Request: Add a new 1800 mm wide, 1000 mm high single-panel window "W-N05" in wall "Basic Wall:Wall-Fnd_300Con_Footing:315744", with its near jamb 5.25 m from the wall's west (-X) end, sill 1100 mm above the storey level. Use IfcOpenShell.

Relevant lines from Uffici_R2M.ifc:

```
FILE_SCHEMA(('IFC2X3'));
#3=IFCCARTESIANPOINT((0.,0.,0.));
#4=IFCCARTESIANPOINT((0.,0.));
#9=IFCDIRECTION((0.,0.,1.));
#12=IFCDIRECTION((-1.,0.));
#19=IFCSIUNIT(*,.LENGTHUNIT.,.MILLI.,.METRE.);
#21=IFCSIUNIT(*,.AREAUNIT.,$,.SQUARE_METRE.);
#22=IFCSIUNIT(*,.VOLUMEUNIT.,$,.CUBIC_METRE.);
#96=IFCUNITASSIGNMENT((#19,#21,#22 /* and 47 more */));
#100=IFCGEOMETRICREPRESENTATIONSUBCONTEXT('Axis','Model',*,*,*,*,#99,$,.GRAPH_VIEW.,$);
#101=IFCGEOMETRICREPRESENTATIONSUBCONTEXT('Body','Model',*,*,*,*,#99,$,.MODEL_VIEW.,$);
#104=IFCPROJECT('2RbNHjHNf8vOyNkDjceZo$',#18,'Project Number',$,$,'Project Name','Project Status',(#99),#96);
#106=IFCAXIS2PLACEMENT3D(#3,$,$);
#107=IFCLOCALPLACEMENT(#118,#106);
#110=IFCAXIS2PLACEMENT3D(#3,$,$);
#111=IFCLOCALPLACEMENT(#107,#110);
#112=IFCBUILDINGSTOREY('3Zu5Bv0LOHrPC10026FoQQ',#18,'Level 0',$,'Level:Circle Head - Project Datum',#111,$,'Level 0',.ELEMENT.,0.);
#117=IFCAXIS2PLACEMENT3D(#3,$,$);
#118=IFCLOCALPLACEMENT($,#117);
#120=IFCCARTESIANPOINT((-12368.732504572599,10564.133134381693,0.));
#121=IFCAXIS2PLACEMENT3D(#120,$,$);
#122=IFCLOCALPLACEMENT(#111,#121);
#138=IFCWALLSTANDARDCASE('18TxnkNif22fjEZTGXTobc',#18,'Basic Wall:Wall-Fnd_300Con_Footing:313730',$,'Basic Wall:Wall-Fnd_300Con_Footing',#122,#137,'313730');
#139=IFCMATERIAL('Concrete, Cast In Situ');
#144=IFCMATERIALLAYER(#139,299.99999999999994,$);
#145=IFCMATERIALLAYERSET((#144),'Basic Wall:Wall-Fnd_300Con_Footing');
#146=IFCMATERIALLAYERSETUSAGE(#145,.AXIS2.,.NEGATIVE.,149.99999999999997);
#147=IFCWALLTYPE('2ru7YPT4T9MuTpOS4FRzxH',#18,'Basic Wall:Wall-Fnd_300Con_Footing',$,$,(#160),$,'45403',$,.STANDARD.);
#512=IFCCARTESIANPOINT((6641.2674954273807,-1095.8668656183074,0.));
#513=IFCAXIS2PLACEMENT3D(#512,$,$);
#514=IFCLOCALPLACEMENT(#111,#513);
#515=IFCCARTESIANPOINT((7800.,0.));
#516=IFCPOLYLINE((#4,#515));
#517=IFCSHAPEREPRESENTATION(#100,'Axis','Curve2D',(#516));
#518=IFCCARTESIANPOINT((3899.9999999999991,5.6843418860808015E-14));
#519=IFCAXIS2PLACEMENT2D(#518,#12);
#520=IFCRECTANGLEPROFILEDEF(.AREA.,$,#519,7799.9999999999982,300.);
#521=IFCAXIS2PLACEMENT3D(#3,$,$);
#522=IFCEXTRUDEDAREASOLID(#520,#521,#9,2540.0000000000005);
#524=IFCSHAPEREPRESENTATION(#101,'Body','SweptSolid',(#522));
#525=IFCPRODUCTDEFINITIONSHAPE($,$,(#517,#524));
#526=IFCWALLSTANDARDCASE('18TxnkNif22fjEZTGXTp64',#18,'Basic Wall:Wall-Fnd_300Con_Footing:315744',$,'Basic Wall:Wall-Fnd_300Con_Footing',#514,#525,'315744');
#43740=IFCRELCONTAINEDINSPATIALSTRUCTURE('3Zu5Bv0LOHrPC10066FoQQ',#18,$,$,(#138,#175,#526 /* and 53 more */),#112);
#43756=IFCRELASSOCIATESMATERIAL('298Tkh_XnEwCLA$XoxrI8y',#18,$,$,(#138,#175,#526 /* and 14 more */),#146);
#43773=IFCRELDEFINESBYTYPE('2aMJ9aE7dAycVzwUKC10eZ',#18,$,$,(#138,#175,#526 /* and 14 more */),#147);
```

```python
import numpy as np
import ifcopenshell
import ifcopenshell.api.feature
import ifcopenshell.api.geometry
import ifcopenshell.api.root
import ifcopenshell.api.spatial
import ifcopenshell.api.type
import ifcopenshell.geom
import ifcopenshell.util.element
import ifcopenshell.util.placement
import ifcopenshell.util.representation
import ifcopenshell.util.shape
import ifcopenshell.util.unit

model = ifcopenshell.open("Uffici_R2M.ifc")
unit_scale = ifcopenshell.util.unit.calculate_unit_scale(model)
settings = ifcopenshell.geom.settings()


def volume(element):
    """Net volume in cubic metres, openings subtracted."""
    shape = ifcopenshell.geom.create_shape(settings, element)
    return ifcopenshell.util.shape.get_volume(shape.geometry)


wall = model.by_guid("18TxnkNif22fjEZTGXTp64")
storey = ifcopenshell.util.element.get_container(wall, ifc_class="IfcBuildingStorey")
context = ifcopenshell.util.representation.get_context(model, "Model", "Body", "MODEL_VIEW")
before = volume(wall)

width, height, from_end, sill = 1.8, 1, 5.25, 1.1  # metres

# The wall runs along its own X axis, and the end named is its -X end.
wall_shape = ifcopenshell.geom.create_shape(settings, wall)
x, y, z = ifcopenshell.util.shape.get_vertices(wall_shape.geometry).T
start = x.min() + from_end
face, thickness = float(y.min()), float(y.max() - y.min())
wall_matrix = ifcopenshell.util.placement.get_local_placement(wall.ObjectPlacement)
level = ifcopenshell.util.placement.get_local_placement(storey.ObjectPlacement)[2, 3]


def in_wall(x, y):
    """Placement at x, y metres in the wall's axes, at sill height."""
    matrix = wall_matrix.copy()
    matrix[:, 3] = wall_matrix @ np.array([x / unit_scale, y / unit_scale, 0.0, 1.0])
    matrix[2, 3] = level + sill / unit_scale
    return matrix


# Opening: a box that overshoots both wall faces by 50 mm.
opening = ifcopenshell.api.root.create_entity(model, ifc_class="IfcOpeningElement")
box = ifcopenshell.api.geometry.add_wall_representation(
    model, context=context, length=width, height=height, thickness=thickness + 0.1
)
ifcopenshell.api.geometry.assign_representation(model, product=opening, representation=box)
ifcopenshell.api.geometry.edit_object_placement(model, product=opening, matrix=in_wall(start, face - 0.05), is_si=False)
ifcopenshell.api.feature.add_feature(model, feature=opening, element=wall)

window = ifcopenshell.api.root.create_entity(model, ifc_class="IfcWindow", name="W-N05")
window.OverallWidth, window.OverallHeight = width / unit_scale, height / unit_scale
body = ifcopenshell.api.geometry.add_window_representation(
    model,
    context=context,
    overall_width=window.OverallWidth,
    overall_height=window.OverallHeight,
    partition_type="SINGLE_PANEL",
)
ifcopenshell.api.geometry.assign_representation(model, product=window, representation=body)
ifcopenshell.api.spatial.assign_container(model, products=[window], relating_structure=storey)
fills = ifcopenshell.api.feature.add_filling(model, opening=opening, element=window)
fills.OwnerHistory = window.OwnerHistory  # required in IFC2X3

# IFC2X3 keeps the operation on the window style.
style = ifcopenshell.api.root.create_entity(model, ifc_class="IfcWindowStyle", name="W-N05")
style.OperationType, style.ConstructionType = "SINGLE_PANEL", "NOTDEFINED"
style.ParameterTakesPrecedence = style.Sizeable = False
ifcopenshell.api.type.assign_type(model, related_objects=[window], relating_type=style)

# Centre the window in the wall's thickness.
ifcopenshell.api.geometry.edit_object_placement(model, product=window, matrix=in_wall(start, face), is_si=False)
window_shape = ifcopenshell.geom.create_shape(settings, window)
depth = ifcopenshell.util.shape.get_vertices(window_shape.geometry)[:, 1]
offset = face + thickness / 2 - (depth.min() + depth.max()) / 2
ifcopenshell.api.geometry.edit_object_placement(model, product=window, matrix=in_wall(start, offset), is_si=False)

after = volume(wall)

print(f"wall volume {before:.3f} -> {after:.3f} m3")

model.write("Uffici_R2M-out.ifc")
```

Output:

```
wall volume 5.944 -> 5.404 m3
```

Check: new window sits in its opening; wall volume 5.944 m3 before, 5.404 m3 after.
